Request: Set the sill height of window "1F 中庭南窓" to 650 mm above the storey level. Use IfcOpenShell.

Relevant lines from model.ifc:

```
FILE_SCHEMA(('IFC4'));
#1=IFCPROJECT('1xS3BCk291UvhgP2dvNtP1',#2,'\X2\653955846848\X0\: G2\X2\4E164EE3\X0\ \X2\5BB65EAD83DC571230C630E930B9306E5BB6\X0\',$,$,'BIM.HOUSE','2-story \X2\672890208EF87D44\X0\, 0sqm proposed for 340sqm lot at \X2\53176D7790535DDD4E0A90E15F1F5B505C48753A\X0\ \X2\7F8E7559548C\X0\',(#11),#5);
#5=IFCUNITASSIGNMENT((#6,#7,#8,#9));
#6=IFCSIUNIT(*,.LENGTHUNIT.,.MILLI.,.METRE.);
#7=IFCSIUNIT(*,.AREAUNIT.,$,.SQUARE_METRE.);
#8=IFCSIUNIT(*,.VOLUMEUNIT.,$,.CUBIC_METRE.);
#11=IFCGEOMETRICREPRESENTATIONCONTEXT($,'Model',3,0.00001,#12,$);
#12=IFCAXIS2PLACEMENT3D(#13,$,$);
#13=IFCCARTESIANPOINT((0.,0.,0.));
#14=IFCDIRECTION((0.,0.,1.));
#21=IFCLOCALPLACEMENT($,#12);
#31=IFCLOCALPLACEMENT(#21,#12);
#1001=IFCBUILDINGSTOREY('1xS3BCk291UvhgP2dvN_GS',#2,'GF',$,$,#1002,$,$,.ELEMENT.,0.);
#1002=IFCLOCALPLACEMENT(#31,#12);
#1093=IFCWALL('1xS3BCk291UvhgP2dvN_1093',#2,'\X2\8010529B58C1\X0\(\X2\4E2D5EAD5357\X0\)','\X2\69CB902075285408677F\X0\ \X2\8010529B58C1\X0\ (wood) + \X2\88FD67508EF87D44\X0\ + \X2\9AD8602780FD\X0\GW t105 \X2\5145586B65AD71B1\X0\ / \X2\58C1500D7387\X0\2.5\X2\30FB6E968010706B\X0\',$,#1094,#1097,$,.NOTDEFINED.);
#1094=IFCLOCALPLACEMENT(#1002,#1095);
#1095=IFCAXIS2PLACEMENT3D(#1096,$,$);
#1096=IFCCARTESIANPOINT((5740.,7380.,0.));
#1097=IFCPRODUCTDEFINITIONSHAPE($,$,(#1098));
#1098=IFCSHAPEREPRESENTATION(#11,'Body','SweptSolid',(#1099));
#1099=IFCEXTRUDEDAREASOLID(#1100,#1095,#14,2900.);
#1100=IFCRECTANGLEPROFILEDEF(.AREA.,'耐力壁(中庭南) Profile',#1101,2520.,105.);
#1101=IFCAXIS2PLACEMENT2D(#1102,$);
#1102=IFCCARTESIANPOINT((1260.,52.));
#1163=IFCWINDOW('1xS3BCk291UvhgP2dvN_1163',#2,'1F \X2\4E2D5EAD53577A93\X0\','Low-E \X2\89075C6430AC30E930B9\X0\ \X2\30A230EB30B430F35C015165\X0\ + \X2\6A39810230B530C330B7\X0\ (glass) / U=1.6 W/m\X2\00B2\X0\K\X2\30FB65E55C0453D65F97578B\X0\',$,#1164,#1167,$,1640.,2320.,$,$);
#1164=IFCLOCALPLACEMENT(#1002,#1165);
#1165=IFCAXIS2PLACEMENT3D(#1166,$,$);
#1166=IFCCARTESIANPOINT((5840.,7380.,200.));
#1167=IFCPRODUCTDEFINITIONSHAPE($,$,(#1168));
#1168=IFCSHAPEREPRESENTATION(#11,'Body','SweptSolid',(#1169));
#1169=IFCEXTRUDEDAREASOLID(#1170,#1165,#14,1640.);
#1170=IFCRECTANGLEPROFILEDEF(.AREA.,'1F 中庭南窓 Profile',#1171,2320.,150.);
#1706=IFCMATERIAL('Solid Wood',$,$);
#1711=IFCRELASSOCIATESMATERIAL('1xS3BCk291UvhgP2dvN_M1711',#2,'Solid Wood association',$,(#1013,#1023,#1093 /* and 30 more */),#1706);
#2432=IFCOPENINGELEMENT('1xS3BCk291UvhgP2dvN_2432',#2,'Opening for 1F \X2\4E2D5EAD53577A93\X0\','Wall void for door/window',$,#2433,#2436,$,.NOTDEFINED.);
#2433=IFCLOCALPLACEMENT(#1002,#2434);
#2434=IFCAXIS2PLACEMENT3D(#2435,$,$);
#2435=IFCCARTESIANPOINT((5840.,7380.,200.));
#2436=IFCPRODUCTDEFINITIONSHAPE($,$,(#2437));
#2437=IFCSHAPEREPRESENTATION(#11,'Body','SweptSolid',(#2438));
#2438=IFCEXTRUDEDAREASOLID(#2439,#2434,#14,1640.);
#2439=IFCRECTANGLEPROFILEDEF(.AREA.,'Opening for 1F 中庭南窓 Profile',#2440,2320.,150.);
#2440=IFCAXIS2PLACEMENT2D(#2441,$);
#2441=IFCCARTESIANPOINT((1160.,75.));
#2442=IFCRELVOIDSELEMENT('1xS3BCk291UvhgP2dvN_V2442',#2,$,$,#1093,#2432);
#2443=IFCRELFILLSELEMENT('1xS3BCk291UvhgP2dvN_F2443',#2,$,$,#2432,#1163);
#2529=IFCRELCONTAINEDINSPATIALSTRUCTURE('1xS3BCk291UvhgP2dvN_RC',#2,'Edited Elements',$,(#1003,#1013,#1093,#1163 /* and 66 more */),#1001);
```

```python
import numpy as np
import ifcopenshell
import ifcopenshell.api.geometry
import ifcopenshell.geom
import ifcopenshell.util.element
import ifcopenshell.util.placement
import ifcopenshell.util.shape
import ifcopenshell.util.unit

model = ifcopenshell.open("model.ifc")
unit_scale = ifcopenshell.util.unit.calculate_unit_scale(model)

window = model.by_guid("1xS3BCk291UvhgP2dvN_1163")
opening = window.FillsVoids[0].RelatingOpeningElement
storey = ifcopenshell.util.element.get_container(window, ifc_class="IfcBuildingStorey")
level = ifcopenshell.util.placement.get_local_placement(storey.ObjectPlacement)[2, 3]

# The opening's origin need not be at the sill, so measure its lowest point.
shape = ifcopenshell.geom.create_shape(ifcopenshell.geom.settings(), opening)
bottom = ifcopenshell.util.shape.get_shape_bottom_elevation(shape, shape.geometry) / unit_scale
dz = level + 0.65 / unit_scale - bottom

shift = np.array([0.0, 0.0, dz])
# The window is not placed relative to its opening, so move both.
for product in (opening, window):
    matrix = ifcopenshell.util.placement.get_local_placement(product.ObjectPlacement)
    matrix[:3, 3] += shift
    ifcopenshell.api.geometry.edit_object_placement(model, product=product, matrix=matrix, is_si=False)

print(f"moved by {dz * unit_scale:+.3f} m")

model.write("model_edited.ifc")
```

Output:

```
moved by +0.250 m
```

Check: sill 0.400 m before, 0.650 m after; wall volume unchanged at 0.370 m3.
